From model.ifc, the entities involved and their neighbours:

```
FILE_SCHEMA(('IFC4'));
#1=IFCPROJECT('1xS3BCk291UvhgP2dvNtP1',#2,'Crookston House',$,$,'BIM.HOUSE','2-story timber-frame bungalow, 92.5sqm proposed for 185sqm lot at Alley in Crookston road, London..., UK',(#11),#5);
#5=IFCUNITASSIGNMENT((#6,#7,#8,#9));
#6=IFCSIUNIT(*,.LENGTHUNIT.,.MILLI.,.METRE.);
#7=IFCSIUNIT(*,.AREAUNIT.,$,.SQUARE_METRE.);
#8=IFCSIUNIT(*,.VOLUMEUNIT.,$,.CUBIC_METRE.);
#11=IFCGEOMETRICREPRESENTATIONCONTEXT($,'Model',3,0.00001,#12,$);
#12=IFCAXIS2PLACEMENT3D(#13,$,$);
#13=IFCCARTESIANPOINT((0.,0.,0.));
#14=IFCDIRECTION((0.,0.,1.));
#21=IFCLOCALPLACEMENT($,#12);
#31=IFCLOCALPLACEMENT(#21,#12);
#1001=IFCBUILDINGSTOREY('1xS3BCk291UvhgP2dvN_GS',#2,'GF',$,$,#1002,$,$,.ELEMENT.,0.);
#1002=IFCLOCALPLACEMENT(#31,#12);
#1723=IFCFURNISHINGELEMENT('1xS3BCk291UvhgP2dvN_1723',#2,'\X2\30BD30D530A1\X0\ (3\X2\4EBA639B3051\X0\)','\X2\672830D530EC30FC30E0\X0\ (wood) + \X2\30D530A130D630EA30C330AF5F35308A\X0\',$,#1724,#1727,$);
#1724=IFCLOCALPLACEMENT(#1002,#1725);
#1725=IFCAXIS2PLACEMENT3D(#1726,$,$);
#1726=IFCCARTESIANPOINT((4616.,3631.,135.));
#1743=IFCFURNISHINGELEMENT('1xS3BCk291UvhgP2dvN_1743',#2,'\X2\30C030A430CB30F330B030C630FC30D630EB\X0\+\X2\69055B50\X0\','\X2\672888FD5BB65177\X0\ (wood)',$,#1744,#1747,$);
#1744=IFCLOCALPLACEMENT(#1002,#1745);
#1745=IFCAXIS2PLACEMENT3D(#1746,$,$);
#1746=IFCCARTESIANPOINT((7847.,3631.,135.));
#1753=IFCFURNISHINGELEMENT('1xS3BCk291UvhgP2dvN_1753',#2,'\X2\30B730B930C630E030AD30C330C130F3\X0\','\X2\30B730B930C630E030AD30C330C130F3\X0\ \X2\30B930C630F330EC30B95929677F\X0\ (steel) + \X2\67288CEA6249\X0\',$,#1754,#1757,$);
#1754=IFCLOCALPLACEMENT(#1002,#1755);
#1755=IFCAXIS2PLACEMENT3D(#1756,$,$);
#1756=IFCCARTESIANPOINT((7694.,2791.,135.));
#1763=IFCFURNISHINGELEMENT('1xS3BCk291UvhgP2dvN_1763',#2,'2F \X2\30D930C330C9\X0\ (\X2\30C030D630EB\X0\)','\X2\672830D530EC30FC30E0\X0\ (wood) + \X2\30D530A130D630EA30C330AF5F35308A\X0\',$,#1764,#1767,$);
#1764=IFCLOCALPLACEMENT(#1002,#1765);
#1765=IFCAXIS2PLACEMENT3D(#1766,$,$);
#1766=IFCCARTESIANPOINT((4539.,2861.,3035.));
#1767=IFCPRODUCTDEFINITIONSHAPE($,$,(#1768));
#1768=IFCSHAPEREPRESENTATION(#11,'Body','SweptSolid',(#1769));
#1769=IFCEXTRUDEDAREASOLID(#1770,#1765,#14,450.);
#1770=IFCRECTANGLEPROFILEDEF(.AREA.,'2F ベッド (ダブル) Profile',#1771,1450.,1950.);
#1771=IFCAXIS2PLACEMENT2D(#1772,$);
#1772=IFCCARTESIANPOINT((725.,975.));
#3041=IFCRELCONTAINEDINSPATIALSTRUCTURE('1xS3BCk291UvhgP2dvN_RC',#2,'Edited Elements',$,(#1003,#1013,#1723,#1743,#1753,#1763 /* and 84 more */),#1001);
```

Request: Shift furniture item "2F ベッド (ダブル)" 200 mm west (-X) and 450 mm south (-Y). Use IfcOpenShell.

```python
import ifcopenshell
import ifcopenshell.api.geometry
import ifcopenshell.util.placement
import ifcopenshell.util.unit

model = ifcopenshell.open("model.ifc")
unit_scale = ifcopenshell.util.unit.calculate_unit_scale(model)

item = model.by_id(1763)
matrix = ifcopenshell.util.placement.get_local_placement(item.ObjectPlacement)
matrix[0, 3] -= 0.2 / unit_scale
matrix[1, 3] -= 0.45 / unit_scale
ifcopenshell.api.geometry.edit_object_placement(model, product=item, matrix=matrix, is_si=False)

print(ifcopenshell.util.placement.get_local_placement(item.ObjectPlacement).round(3) + 0.0)

model.write("model_edited.ifc")
```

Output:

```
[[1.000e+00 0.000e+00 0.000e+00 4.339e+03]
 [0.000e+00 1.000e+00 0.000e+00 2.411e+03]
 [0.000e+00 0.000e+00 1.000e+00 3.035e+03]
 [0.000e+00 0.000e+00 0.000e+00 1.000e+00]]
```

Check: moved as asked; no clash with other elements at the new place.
